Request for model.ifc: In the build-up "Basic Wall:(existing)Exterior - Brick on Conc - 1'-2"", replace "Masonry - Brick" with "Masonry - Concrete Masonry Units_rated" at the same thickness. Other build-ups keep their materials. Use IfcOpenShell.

First a look at what the model holds.

```python
import ifcopenshell
import ifcopenshell.util.element

model = ifcopenshell.open("model.ifc")
print(model.schema)
for layer_set in model.by_type("IfcMaterialLayerSet"):
    if layer_set.LayerSetName == 'Basic Wall:(existing)Exterior - Brick on Conc - 1\'-2"':
        for layer in layer_set.MaterialLayers:
            print(layer.id(), layer.Material and layer.Material.Name, layer.LayerThickness, sep=" | ")
        print(len(ifcopenshell.util.element.get_elements_by_material(model, layer_set)), "elements and types use it")
print(sorted(m.Name for m in model.by_type("IfcMaterial") if m.Name)[:60])
```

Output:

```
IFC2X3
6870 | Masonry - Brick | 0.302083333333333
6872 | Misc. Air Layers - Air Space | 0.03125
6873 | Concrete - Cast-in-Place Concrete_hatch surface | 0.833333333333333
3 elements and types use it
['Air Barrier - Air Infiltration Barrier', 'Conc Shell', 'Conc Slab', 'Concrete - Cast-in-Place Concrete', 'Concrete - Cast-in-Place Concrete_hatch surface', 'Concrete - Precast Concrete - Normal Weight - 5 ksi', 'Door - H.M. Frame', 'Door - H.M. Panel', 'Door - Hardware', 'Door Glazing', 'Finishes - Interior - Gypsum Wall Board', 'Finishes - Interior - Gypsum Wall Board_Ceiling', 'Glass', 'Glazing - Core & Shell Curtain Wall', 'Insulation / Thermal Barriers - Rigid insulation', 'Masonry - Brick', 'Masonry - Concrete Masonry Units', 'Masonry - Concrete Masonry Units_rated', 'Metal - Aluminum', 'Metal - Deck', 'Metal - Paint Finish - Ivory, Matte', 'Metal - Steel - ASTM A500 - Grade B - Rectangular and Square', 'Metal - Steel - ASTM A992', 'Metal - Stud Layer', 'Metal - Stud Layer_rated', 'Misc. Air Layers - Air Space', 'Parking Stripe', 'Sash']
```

```python
import ifcopenshell
import ifcopenshell.api.material

model = ifcopenshell.open("model.ifc")

layer_set = next(s for s in model.by_type("IfcMaterialLayerSet") if s.LayerSetName == 'Basic Wall:(existing)Exterior - Brick on Conc - 1\'-2"')
layer = next(l for l in layer_set.MaterialLayers if l.Material and l.Material.Name == "Masonry - Brick")
material = next(m for m in model.by_type("IfcMaterial") if m.Name == "Masonry - Concrete Masonry Units_rated")

# Point this one layer at the other material; renaming the old one would change it everywhere.
ifcopenshell.api.material.edit_layer(model, layer=layer, attributes={}, material=material)

print([l.Material.Name if l.Material else None for l in layer_set.MaterialLayers])

model.write("model_edited.ifc")
```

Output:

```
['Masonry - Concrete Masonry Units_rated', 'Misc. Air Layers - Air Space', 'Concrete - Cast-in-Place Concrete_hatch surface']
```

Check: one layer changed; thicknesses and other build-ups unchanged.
